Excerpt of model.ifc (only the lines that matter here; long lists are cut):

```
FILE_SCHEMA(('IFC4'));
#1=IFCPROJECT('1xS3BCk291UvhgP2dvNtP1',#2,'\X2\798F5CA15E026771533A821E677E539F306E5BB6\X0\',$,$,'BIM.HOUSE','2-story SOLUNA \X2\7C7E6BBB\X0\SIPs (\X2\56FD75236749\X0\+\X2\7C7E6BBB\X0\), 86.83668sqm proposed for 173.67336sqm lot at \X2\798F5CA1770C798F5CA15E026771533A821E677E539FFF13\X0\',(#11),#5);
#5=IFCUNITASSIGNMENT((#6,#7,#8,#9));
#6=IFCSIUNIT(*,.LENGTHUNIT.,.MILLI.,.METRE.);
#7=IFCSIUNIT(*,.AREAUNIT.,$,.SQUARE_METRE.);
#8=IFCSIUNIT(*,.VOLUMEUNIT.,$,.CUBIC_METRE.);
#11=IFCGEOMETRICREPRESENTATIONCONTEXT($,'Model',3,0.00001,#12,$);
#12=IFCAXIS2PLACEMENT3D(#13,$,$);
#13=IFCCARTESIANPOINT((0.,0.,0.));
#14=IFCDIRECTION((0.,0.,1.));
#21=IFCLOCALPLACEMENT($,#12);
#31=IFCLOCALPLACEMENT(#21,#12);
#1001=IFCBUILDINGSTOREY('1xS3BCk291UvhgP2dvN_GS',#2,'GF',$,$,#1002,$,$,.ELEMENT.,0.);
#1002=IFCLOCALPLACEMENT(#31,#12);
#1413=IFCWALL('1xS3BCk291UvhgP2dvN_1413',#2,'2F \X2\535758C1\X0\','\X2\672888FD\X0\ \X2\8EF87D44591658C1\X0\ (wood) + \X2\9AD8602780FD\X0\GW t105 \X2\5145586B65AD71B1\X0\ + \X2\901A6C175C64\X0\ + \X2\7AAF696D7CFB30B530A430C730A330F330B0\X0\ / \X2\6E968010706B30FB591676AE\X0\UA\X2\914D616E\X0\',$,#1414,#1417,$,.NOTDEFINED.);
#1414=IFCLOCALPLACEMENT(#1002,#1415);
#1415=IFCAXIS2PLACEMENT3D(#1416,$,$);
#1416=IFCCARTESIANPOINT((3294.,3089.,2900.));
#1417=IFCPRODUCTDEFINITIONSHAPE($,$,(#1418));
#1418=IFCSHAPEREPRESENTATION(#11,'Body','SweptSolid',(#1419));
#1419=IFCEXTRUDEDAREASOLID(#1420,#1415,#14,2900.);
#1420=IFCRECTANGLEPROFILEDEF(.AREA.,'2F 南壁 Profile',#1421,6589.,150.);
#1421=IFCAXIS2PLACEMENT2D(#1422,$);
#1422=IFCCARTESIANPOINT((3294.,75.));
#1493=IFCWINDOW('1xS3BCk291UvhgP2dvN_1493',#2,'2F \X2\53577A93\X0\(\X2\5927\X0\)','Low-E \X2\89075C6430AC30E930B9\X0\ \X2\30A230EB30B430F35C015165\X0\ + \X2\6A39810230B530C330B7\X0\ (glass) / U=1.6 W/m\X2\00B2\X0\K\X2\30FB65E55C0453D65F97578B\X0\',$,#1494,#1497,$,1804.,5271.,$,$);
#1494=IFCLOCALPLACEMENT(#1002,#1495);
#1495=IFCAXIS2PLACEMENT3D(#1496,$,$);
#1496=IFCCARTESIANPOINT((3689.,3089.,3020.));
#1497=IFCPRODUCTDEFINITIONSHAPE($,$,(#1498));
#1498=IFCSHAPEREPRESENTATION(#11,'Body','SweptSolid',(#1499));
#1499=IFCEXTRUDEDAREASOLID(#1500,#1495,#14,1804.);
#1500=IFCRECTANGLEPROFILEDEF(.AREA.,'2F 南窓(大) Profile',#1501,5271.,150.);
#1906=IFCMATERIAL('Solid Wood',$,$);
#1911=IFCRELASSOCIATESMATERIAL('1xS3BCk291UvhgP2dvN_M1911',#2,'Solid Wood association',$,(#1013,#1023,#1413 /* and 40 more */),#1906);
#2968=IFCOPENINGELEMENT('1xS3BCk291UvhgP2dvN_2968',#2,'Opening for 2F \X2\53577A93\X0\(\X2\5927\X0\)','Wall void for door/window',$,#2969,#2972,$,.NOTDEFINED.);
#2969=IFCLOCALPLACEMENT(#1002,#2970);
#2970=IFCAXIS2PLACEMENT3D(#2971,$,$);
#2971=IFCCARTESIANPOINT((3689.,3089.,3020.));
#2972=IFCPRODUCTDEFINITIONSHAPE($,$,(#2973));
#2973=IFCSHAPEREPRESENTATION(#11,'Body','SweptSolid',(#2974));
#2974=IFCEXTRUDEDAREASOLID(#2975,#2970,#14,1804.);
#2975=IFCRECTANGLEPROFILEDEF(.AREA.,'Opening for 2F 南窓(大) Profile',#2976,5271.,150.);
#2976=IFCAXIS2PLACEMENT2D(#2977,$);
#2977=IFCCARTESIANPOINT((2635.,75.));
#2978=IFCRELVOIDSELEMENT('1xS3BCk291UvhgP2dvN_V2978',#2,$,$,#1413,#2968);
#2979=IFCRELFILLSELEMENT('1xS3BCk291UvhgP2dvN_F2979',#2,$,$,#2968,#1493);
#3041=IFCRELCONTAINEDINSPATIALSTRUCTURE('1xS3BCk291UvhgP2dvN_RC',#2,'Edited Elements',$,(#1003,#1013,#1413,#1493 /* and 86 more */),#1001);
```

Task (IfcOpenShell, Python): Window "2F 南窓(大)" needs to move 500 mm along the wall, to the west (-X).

```python
import ifcopenshell
import ifcopenshell.api.geometry
import ifcopenshell.util.placement
import ifcopenshell.util.unit

model = ifcopenshell.open("model.ifc")
unit_scale = ifcopenshell.util.unit.calculate_unit_scale(model)

window = model.by_guid("1xS3BCk291UvhgP2dvN_1493")
opening = window.FillsVoids[0].RelatingOpeningElement
wall = opening.VoidsElements[0].RelatingBuildingElement

wall_matrix = ifcopenshell.util.placement.get_local_placement(wall.ObjectPlacement)
shift = wall_matrix[:3, 0] * -0.5 / unit_scale
before = ifcopenshell.util.placement.get_local_placement(window.ObjectPlacement)[:3, 3].copy()

# The window is not placed relative to its opening, so move both.
for product in (opening, window):
    matrix = ifcopenshell.util.placement.get_local_placement(product.ObjectPlacement)
    matrix[:3, 3] += shift
    ifcopenshell.api.geometry.edit_object_placement(model, product=product, matrix=matrix, is_si=False)

after = ifcopenshell.util.placement.get_local_placement(window.ObjectPlacement)[:3, 3]
print("window moved by", (after - before).round(3) + 0.0)

model.write("model_updated.ifc")
```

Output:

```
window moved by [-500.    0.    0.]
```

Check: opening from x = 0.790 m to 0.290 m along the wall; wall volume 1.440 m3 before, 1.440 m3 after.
